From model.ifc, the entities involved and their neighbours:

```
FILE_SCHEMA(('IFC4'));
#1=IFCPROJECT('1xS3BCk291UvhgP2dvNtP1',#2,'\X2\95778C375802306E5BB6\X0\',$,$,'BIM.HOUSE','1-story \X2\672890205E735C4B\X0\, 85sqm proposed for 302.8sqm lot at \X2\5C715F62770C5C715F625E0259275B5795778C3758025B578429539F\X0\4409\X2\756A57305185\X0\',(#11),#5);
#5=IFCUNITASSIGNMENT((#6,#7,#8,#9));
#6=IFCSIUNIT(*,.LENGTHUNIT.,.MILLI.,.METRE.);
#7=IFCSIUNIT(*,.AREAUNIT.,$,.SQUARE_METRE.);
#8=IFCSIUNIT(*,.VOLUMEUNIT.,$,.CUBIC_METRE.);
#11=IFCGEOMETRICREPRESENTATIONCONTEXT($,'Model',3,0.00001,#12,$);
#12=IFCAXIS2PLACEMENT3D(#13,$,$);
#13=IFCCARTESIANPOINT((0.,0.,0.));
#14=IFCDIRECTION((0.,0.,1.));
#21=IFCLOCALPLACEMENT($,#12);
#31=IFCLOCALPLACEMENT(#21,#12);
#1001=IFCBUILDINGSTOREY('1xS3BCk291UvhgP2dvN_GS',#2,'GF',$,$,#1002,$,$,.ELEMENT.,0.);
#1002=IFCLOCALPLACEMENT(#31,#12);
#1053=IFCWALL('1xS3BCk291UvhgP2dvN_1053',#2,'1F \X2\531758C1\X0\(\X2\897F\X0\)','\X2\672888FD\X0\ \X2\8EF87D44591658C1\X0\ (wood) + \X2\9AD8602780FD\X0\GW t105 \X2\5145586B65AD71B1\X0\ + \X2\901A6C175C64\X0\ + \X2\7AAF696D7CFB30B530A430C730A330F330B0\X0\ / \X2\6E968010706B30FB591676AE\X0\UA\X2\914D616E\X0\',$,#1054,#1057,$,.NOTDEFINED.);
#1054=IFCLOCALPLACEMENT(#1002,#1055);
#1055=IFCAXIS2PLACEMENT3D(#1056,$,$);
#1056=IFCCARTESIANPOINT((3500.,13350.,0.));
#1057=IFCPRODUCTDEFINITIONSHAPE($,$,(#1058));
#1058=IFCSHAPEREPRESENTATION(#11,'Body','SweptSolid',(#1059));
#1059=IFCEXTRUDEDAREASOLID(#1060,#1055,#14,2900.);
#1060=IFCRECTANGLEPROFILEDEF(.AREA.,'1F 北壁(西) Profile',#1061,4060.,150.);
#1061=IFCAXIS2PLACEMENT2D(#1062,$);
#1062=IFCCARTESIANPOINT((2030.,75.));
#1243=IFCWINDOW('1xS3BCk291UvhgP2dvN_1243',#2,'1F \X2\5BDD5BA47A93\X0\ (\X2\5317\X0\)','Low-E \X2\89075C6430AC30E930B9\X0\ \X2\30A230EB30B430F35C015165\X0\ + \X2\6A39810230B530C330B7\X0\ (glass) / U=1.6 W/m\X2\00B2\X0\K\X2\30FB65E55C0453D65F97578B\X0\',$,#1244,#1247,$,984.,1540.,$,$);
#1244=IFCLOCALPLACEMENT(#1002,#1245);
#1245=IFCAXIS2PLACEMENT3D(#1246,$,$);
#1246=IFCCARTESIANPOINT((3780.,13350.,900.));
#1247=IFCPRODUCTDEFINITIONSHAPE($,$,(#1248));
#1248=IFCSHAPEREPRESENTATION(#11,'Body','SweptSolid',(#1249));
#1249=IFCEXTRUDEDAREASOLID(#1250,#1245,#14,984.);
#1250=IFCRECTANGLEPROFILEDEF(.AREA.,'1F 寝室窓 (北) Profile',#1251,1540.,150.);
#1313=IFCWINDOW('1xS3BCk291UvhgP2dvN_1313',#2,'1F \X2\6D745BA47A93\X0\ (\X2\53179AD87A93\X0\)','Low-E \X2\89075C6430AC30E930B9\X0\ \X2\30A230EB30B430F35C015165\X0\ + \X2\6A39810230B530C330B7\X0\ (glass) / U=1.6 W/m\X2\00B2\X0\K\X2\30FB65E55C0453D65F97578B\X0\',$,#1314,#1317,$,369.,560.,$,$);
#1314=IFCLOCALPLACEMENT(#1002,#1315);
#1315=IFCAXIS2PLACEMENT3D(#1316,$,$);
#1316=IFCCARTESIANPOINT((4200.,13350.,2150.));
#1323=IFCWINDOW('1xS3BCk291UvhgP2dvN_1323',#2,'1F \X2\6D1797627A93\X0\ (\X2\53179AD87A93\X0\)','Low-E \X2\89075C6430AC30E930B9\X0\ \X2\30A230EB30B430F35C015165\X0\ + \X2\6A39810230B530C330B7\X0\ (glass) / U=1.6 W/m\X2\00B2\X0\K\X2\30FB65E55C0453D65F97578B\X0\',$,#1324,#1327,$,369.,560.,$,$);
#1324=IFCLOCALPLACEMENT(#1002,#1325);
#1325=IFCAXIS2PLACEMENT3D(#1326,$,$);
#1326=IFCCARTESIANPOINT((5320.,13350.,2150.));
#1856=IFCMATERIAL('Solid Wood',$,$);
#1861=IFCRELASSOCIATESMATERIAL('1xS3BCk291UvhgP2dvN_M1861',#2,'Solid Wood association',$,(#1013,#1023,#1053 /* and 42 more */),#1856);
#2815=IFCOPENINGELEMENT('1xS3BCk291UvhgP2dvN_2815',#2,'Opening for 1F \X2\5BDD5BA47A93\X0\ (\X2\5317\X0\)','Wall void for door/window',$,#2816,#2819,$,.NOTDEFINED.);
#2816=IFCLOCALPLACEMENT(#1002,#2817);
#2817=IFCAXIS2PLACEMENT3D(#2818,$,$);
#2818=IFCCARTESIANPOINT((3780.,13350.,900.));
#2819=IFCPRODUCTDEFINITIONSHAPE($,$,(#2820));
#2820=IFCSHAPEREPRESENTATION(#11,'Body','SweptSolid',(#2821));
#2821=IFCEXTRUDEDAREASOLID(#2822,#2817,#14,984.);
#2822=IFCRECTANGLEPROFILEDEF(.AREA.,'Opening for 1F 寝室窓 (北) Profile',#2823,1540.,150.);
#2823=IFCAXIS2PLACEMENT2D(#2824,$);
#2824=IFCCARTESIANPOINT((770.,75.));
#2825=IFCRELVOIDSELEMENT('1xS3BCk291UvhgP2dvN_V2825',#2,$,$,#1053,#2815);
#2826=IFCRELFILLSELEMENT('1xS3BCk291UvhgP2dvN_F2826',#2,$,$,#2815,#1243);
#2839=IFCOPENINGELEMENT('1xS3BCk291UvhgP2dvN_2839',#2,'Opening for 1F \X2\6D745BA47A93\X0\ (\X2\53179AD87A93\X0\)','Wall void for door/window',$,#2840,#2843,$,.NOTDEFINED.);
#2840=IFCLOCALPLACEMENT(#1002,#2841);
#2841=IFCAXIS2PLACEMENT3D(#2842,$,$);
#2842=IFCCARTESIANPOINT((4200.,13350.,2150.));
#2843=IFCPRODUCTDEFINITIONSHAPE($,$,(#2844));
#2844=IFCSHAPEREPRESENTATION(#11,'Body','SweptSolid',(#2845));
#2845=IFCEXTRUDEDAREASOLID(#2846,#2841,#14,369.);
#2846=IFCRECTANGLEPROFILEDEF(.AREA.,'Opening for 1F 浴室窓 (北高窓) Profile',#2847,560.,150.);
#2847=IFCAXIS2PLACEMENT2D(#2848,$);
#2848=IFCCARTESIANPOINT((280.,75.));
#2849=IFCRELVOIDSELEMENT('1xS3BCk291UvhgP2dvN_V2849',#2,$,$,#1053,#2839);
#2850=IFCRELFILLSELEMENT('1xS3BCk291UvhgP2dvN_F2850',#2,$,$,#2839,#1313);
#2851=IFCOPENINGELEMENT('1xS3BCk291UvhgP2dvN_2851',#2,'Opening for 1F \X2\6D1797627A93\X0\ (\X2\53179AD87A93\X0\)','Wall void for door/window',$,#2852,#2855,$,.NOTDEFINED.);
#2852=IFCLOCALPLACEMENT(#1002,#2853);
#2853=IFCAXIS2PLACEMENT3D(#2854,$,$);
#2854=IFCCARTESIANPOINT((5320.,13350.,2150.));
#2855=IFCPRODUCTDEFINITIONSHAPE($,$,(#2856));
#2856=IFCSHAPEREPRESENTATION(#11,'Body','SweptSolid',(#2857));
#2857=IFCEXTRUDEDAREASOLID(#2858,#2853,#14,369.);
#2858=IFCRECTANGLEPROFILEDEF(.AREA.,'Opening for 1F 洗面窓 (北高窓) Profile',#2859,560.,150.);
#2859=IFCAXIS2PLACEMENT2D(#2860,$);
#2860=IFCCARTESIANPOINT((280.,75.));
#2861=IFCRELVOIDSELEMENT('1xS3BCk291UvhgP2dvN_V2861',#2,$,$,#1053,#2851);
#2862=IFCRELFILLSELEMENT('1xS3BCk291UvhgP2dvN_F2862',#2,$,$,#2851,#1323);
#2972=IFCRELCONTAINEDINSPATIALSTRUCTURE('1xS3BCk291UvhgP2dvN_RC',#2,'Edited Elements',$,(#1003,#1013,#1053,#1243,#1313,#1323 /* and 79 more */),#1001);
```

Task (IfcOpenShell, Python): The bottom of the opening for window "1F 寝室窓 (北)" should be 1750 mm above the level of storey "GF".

```python
import numpy as np
import ifcopenshell
import ifcopenshell.api.geometry
import ifcopenshell.geom
import ifcopenshell.util.element
import ifcopenshell.util.placement
import ifcopenshell.util.shape
import ifcopenshell.util.unit

model = ifcopenshell.open("model.ifc")
unit_scale = ifcopenshell.util.unit.calculate_unit_scale(model)

window = model.by_guid("1xS3BCk291UvhgP2dvN_1243")
opening = window.FillsVoids[0].RelatingOpeningElement
storey = ifcopenshell.util.element.get_container(window, ifc_class="IfcBuildingStorey")
level = ifcopenshell.util.placement.get_local_placement(storey.ObjectPlacement)[2, 3]

# The opening's origin need not be at the sill, so measure its lowest point.
shape = ifcopenshell.geom.create_shape(ifcopenshell.geom.settings(), opening)
bottom = ifcopenshell.util.shape.get_shape_bottom_elevation(shape, shape.geometry) / unit_scale
dz = level + 1750.0 - bottom

shift = np.array([0.0, 0.0, dz])
# The window is not placed relative to its opening, so move both.
for product in (opening, window):
    matrix = ifcopenshell.util.placement.get_local_placement(product.ObjectPlacement)
    matrix[:3, 3] += shift
    ifcopenshell.api.geometry.edit_object_placement(model, product=product, matrix=matrix, is_si=False)

print(f"moved by {dz * unit_scale:+.3f} m")

model.write("model_edited.ifc")
```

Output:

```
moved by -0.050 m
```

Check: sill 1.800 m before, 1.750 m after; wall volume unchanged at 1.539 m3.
